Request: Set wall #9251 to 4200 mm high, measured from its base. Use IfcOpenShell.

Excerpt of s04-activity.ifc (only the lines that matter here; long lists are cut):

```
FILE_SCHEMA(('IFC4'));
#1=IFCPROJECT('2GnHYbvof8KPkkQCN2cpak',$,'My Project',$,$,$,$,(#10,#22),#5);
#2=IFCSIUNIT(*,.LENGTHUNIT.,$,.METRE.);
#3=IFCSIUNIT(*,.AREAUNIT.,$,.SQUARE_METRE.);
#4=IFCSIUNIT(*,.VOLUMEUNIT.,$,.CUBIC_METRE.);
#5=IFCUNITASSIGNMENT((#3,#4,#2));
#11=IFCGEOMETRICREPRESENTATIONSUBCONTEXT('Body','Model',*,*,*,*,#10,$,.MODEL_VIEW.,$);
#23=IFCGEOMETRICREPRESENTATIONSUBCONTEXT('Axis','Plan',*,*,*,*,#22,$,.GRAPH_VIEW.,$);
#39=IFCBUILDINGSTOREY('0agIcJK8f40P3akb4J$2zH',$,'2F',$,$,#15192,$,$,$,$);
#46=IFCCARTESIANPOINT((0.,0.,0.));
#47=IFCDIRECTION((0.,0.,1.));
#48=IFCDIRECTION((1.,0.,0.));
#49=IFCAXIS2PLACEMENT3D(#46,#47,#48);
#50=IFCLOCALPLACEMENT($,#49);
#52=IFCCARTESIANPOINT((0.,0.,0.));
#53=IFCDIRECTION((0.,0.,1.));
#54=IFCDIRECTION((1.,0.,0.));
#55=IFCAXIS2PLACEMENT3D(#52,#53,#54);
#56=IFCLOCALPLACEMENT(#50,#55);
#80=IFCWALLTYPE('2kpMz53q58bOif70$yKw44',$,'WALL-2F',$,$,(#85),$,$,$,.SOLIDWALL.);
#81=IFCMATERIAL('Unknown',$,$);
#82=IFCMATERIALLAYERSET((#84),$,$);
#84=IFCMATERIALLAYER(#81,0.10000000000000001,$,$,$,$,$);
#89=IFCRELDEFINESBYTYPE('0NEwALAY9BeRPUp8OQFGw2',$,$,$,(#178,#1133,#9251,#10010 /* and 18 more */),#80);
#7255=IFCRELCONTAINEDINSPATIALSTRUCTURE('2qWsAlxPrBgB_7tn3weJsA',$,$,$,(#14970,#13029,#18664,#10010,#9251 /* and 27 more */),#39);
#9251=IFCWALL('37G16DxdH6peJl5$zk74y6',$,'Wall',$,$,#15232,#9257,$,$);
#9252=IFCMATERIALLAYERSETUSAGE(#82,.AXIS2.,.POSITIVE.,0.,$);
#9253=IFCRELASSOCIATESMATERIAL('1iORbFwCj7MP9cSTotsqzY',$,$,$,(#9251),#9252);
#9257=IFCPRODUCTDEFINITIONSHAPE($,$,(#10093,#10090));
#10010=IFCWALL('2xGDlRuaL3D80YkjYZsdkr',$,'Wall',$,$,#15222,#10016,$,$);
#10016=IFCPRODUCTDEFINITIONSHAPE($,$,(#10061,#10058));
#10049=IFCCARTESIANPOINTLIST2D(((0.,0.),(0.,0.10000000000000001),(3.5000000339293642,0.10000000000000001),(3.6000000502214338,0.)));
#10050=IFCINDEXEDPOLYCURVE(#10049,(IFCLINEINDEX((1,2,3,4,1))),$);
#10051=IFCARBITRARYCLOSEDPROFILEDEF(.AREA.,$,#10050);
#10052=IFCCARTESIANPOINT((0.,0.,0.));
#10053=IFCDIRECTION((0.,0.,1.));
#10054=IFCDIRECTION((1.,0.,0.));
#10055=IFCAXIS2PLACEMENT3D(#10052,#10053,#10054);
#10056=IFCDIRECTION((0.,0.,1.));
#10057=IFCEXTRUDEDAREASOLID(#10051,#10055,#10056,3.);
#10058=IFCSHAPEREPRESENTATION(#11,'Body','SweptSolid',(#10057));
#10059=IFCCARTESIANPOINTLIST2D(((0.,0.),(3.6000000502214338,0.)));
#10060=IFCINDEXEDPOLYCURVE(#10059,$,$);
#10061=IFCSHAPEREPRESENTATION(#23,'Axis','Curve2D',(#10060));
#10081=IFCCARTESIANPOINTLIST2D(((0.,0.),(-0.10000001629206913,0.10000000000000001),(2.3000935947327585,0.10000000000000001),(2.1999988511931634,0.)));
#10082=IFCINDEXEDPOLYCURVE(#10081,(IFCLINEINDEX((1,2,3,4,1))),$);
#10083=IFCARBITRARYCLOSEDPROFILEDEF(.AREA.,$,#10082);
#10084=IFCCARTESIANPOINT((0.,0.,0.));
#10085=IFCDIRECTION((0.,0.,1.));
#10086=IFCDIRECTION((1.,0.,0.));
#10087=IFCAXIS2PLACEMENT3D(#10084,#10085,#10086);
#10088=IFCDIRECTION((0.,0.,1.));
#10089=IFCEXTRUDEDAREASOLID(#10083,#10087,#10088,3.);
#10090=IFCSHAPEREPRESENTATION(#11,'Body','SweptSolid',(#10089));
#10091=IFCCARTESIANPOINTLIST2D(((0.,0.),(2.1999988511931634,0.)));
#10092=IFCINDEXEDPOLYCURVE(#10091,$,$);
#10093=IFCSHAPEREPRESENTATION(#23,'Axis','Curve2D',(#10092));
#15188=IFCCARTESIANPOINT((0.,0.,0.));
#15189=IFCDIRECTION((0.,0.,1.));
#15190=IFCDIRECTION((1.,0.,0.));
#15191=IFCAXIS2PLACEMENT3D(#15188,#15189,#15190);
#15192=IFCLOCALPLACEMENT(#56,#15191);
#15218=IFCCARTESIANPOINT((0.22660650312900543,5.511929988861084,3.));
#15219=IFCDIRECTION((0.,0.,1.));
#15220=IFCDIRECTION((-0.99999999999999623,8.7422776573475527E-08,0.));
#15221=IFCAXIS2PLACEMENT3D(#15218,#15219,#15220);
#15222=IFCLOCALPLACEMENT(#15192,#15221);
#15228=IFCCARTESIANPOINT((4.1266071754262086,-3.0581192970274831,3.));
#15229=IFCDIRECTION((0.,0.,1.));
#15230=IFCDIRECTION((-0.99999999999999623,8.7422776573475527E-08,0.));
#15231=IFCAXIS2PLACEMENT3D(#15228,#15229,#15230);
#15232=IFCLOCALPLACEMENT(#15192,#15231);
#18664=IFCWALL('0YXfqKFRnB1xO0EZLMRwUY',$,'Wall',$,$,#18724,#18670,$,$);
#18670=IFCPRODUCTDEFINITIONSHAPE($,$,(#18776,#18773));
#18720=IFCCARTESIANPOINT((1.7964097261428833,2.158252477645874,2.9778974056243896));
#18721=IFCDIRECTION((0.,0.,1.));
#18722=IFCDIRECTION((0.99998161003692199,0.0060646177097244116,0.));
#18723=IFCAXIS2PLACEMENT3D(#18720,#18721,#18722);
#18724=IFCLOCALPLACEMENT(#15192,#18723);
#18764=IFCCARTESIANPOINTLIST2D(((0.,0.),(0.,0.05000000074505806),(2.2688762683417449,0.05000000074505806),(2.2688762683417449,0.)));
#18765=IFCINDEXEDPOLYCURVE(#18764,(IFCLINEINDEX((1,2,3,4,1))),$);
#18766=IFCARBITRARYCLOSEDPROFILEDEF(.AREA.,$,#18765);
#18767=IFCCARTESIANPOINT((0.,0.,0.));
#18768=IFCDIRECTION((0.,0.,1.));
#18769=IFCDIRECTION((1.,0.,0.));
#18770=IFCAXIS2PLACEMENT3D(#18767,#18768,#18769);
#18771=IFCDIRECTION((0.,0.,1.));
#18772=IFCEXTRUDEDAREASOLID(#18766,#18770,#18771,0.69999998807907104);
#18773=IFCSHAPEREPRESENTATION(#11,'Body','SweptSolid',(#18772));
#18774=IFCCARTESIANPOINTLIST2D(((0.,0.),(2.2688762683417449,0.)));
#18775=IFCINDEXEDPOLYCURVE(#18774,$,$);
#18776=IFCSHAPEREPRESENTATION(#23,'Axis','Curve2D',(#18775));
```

```python
import ifcopenshell
import ifcopenshell.geom
import ifcopenshell.util.representation
import ifcopenshell.util.shape

model = ifcopenshell.open("s04-activity.ifc")
settings = ifcopenshell.geom.settings()


def volume(element):
    """Net volume in cubic metres, openings subtracted."""
    shape = ifcopenshell.geom.create_shape(settings, element)
    return ifcopenshell.util.shape.get_volume(shape.geometry)


wall = model.by_guid("37G16DxdH6peJl5$zk74y6")
before = volume(wall)

body = ifcopenshell.util.representation.get_representation(wall, "Model", "Body")
solid = body.Items[0]
old_height = solid.Depth
solid.Depth = 4.2
after = volume(wall)

print(f"height {old_height:g} -> {solid.Depth:g}, volume {before:.3f} -> {after:.3f} m3")

model.write("s04-activity_v2.ifc")
```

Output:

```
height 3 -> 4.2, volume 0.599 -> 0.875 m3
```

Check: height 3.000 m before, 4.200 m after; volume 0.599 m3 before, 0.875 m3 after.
